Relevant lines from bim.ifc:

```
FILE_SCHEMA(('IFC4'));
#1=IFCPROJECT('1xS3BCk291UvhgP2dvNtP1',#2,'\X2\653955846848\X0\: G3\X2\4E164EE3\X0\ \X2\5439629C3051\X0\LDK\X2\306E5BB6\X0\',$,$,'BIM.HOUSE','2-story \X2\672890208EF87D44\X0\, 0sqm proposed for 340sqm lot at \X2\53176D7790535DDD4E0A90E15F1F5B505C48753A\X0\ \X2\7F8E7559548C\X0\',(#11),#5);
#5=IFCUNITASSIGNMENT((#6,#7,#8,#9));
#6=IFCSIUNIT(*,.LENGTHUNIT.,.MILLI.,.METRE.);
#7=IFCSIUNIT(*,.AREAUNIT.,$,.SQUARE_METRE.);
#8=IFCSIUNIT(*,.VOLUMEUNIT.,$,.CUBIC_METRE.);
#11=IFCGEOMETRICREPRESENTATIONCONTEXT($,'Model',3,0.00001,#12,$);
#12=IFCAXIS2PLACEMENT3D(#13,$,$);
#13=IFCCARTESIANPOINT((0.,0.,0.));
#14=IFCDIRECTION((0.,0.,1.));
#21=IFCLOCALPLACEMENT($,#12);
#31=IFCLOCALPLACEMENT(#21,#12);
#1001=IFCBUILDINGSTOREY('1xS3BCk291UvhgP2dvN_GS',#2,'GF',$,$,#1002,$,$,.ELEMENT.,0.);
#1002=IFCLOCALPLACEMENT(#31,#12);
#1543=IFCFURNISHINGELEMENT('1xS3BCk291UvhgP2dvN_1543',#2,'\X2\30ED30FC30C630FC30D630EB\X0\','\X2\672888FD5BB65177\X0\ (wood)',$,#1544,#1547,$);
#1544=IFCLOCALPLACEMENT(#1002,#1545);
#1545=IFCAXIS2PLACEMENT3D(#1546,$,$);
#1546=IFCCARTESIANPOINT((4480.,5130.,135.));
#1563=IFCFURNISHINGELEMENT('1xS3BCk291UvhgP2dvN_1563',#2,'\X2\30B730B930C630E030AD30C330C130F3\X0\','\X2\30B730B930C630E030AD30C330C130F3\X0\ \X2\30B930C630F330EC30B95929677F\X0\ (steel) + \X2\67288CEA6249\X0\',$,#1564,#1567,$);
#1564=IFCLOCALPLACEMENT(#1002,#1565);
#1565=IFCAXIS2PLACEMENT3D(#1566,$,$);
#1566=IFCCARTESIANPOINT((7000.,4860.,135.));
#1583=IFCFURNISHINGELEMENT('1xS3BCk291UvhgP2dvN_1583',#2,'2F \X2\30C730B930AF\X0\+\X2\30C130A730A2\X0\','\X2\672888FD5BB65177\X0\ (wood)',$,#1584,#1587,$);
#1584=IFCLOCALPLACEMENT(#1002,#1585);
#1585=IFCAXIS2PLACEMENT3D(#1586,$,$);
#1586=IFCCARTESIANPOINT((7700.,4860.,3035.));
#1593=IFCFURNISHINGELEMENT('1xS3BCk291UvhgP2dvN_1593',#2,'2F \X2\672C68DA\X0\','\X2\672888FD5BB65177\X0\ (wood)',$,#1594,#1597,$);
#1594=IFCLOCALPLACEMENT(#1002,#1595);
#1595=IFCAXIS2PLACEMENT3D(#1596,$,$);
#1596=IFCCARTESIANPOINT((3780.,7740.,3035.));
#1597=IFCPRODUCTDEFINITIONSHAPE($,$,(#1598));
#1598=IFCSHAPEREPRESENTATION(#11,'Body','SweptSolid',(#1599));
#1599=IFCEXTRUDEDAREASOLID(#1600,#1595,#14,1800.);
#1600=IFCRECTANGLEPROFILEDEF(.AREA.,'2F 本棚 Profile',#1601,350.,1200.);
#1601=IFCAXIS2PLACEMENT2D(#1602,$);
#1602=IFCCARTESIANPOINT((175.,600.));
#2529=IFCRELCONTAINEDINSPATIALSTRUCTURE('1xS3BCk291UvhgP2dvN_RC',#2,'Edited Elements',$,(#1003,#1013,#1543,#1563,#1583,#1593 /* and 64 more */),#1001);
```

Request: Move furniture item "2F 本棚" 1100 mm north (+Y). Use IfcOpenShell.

```python
import ifcopenshell
import ifcopenshell.api.geometry
import ifcopenshell.util.placement

model = ifcopenshell.open("bim.ifc")

item = model.by_guid("1xS3BCk291UvhgP2dvN_1593")
matrix = ifcopenshell.util.placement.get_local_placement(item.ObjectPlacement)
matrix[1, 3] += 1100.0
ifcopenshell.api.geometry.edit_object_placement(model, product=item, matrix=matrix, is_si=False)

print(ifcopenshell.util.placement.get_local_placement(item.ObjectPlacement).round(3) + 0.0)

model.write("bim-out.ifc")
```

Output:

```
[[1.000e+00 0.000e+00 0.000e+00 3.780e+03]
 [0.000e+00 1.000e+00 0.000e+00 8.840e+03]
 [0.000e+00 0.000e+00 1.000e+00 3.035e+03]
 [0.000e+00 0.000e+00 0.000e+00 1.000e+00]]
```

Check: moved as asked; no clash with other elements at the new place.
